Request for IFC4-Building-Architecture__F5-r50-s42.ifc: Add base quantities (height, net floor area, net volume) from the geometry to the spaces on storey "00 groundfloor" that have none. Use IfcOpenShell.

First a look at what the model holds.

```python
import ifcopenshell
import ifcopenshell.util.element
import ifcopenshell.util.unit

model = ifcopenshell.open("IFC4-Building-Architecture__F5-r50-s42.ifc")
print(model.schema)
for unit_type in ("LENGTHUNIT", "AREAUNIT", "VOLUMEUNIT"):
    print(unit_type, ifcopenshell.util.unit.calculate_unit_scale(model, unit_type))
storey = next(s for s in model.by_type("IfcBuildingStorey") if s.Name == "00 groundfloor")
spaces = [e for e in ifcopenshell.util.element.get_decomposition(storey) if e.is_a("IfcSpace")]
for e in sorted(spaces, key=lambda e: e.id()):
    print(e.id(), e.is_a(), e.Name, list(ifcopenshell.util.element.get_psets(e, qtos_only=True)), sep=" | ")
```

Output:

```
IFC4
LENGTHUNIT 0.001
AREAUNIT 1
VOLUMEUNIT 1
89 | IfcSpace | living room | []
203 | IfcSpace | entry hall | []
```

```python
import ifcopenshell
import ifcopenshell.api.pset
import ifcopenshell.geom
import ifcopenshell.util.element
import ifcopenshell.util.shape
import ifcopenshell.util.unit

model = ifcopenshell.open("IFC4-Building-Architecture__F5-r50-s42.ifc")
unit_scale = ifcopenshell.util.unit.calculate_unit_scale(model)
area_scale = ifcopenshell.util.unit.calculate_unit_scale(model, "AREAUNIT")
volume_scale = ifcopenshell.util.unit.calculate_unit_scale(model, "VOLUMEUNIT")
settings = ifcopenshell.geom.settings()

storey = next(s for s in model.by_type("IfcBuildingStorey") if s.Name == "00 groundfloor")
spaces = [e for e in ifcopenshell.util.element.get_decomposition(storey) if e.is_a("IfcSpace")]

for e in sorted(spaces, key=lambda e: e.id()):
    if ifcopenshell.util.element.get_psets(e, qtos_only=True, should_inherit=False):
        continue
    # Geometry comes back in metres, in the element's own axes.
    shape = ifcopenshell.geom.create_shape(settings, e)
    values = {
        "Height": ifcopenshell.util.shape.get_z(shape.geometry) / unit_scale,
        "NetFloorArea": ifcopenshell.util.shape.get_footprint_area(shape.geometry) / area_scale,
        "NetVolume": ifcopenshell.util.shape.get_volume(shape.geometry) / volume_scale,
    }
    qto = ifcopenshell.api.pset.add_qto(model, product=e, name="Qto_SpaceBaseQuantities")
    ifcopenshell.api.pset.edit_qto(model, qto=qto, properties=values)
    print(e.id(), {k: round(v, 3) for k, v in values.items()})

model.write("IFC4-Building-Architecture__F5-r50-s42_edited.ifc")
```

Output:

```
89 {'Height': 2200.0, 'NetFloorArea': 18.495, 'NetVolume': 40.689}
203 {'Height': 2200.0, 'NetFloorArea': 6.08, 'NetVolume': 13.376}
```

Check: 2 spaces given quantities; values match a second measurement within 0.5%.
